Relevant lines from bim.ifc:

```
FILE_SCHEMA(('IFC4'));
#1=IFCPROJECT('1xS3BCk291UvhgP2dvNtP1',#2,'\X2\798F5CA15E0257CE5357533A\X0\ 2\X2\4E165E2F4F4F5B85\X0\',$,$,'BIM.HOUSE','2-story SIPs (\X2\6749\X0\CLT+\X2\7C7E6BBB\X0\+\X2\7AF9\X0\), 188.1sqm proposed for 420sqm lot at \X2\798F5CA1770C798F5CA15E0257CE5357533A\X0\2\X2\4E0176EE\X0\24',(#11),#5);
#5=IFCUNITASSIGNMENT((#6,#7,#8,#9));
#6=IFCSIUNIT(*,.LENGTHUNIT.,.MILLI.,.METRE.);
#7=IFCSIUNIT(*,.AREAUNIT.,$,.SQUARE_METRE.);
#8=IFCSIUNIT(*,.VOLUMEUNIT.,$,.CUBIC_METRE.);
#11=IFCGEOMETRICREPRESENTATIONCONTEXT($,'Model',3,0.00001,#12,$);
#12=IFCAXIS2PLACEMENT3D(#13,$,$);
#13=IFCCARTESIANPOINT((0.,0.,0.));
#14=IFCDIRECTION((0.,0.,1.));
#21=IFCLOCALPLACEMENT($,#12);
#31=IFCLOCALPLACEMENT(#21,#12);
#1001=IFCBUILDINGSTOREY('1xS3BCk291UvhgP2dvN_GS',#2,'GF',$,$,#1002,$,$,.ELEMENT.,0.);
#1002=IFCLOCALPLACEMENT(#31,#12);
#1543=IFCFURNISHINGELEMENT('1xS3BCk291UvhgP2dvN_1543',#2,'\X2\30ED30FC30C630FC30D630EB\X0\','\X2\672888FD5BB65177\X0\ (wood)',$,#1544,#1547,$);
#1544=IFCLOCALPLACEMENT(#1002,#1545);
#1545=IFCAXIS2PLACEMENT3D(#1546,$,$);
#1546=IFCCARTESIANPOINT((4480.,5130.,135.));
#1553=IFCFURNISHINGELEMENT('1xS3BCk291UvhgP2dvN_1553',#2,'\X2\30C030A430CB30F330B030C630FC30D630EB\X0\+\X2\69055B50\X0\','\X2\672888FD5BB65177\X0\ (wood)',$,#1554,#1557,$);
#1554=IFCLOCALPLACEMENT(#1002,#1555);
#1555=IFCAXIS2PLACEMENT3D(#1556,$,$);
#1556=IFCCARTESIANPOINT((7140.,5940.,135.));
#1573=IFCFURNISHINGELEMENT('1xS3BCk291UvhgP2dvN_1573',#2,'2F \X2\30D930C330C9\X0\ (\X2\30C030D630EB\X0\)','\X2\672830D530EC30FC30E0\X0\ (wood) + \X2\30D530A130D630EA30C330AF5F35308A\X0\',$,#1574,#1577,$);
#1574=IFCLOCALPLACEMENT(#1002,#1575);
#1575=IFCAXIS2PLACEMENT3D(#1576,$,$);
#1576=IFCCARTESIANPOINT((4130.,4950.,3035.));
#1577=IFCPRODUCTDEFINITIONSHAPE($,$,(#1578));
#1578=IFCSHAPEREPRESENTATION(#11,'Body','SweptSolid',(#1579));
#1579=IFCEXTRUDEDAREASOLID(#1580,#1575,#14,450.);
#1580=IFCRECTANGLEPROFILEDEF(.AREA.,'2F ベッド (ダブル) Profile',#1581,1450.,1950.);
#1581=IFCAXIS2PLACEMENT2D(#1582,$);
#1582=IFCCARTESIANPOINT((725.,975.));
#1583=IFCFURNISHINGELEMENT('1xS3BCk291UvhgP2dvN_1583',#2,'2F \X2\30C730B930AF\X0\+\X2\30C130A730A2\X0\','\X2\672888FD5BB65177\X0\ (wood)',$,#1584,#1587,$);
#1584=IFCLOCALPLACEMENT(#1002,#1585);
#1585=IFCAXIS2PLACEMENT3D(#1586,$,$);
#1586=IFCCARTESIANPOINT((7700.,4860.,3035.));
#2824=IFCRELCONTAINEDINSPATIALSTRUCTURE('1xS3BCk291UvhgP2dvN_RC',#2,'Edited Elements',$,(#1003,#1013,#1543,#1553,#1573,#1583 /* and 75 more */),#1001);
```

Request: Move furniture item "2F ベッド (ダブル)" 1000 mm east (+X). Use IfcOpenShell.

```python
import ifcopenshell
import ifcopenshell.api.geometry
import ifcopenshell.util.placement
import ifcopenshell.util.unit

model = ifcopenshell.open("bim.ifc")
unit_scale = ifcopenshell.util.unit.calculate_unit_scale(model)

item = model.by_id(1573)
matrix = ifcopenshell.util.placement.get_local_placement(item.ObjectPlacement)
matrix[0, 3] += 1 / unit_scale
ifcopenshell.api.geometry.edit_object_placement(model, product=item, matrix=matrix, is_si=False)

print(ifcopenshell.util.placement.get_local_placement(item.ObjectPlacement).round(3) + 0.0)

model.write("bim_rev.ifc")
```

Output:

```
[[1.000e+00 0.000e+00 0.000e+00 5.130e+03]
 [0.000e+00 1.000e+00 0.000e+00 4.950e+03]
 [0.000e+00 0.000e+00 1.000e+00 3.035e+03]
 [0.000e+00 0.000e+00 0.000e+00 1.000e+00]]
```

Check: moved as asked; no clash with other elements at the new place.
